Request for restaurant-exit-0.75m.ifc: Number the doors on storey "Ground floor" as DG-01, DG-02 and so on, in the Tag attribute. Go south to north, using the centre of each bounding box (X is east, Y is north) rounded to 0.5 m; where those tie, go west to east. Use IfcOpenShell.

First a look at what the model holds.

```python
import ifcopenshell
import ifcopenshell.util.element
import ifcopenshell.util.placement

model = ifcopenshell.open("restaurant-exit-0.75m.ifc")
print(model.schema)
storey = next(s for s in model.by_type("IfcBuildingStorey") if s.Name == "Ground floor")
doors = [e for e in ifcopenshell.util.element.get_decomposition(storey) if e.is_a("IfcDoor")]
for e in sorted(doors, key=lambda e: e.id()):
    origin = ifcopenshell.util.placement.get_local_placement(e.ObjectPlacement)[:3, 3]
    print(e.id(), e.Tag, e.Name, origin.round(2) + 0.0, sep=" | ")
```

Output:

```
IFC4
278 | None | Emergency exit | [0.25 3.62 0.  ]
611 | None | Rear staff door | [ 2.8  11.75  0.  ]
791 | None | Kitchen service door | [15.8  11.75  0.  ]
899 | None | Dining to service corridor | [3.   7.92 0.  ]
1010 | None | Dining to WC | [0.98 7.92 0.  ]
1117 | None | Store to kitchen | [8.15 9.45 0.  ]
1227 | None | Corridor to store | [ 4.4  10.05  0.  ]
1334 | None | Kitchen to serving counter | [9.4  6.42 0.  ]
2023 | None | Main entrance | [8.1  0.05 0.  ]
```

```python
import ifcopenshell
import ifcopenshell.geom
import ifcopenshell.util.element
import ifcopenshell.util.shape

model = ifcopenshell.open("restaurant-exit-0.75m.ifc")
settings = ifcopenshell.geom.settings()
settings.set("use-world-coords", True)


def centre(element):
    shape = ifcopenshell.geom.create_shape(settings, element)
    return ifcopenshell.util.shape.get_bbox_centroid(shape.geometry)


storey = next(s for s in model.by_type("IfcBuildingStorey") if s.Name == "Ground floor")
doors = [e for e in ifcopenshell.util.element.get_decomposition(storey) if e.is_a("IfcDoor")]

# Insertion points can sit at a corner or the storey origin, so sort by the geometry (in metres).
centres = {e: centre(e) for e in doors}
doors.sort(key=lambda e: (round(centres[e][1] / 0.5), centres[e][0]))

for i, e in enumerate(doors, start=1):
    number = f"DG-{i:02d}"
    e.Tag = number
    print(e.id(), number)

model.write("restaurant-exit-0.75m_v2.ifc")
```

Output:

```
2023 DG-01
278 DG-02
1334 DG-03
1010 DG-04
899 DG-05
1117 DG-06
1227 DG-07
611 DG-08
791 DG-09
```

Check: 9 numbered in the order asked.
